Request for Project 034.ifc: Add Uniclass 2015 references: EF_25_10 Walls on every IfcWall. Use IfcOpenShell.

First a look at what the model holds.

```python
import ifcopenshell

model = ifcopenshell.open("Project 034.ifc")
print(model.schema)
print("classifications:", [c.Name for c in model.by_type("IfcClassification")])
for ifc_class in ("IfcDoor", "IfcRoof", "IfcStair", "IfcWall", "IfcWindow"):
    print(ifc_class, len(model.by_type(ifc_class)))
```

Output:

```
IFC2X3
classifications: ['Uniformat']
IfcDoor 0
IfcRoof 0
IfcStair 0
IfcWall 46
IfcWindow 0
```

```python
import ifcopenshell
import ifcopenshell.api.classification

model = ifcopenshell.open("Project 034.ifc")

# IFC2X3 requires Source and Edition and has no link from the project to the system.
system = model.create_entity("IfcClassification", Source="NBS", Edition="2015", Name="Uniclass 2015")

codes = {
    "IfcWall": ("EF_25_10", "Walls"),
}
for ifc_class, (code, name) in codes.items():
    products = model.by_type(ifc_class)
    ifcopenshell.api.classification.add_reference(
        model, products=products, classification=system, identification=code, name=name
    )
    print(code, len(products))

model.write("Project 034_updated.ifc")
```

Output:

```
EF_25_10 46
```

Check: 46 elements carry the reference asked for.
